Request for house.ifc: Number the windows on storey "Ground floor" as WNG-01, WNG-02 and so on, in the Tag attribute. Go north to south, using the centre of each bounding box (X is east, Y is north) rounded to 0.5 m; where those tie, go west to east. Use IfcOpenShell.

First a look at what the model holds.

```python
import ifcopenshell
import ifcopenshell.util.element
import ifcopenshell.util.placement

model = ifcopenshell.open("house.ifc")
print(model.schema)
storey = next(s for s in model.by_type("IfcBuildingStorey") if s.Name == "Ground floor")
windows = [e for e in ifcopenshell.util.element.get_decomposition(storey) if e.is_a("IfcWindow")]
for e in sorted(windows, key=lambda e: e.id()):
    origin = ifcopenshell.util.placement.get_local_placement(e.ObjectPlacement)[:3, 3]
    print(e.id(), e.Tag, e.Name, origin.round(2) + 0.0, sep=" | ")
```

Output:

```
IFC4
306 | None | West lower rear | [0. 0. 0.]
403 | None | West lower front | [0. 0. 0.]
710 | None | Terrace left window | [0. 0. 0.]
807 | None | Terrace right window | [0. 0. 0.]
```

```python
import ifcopenshell
import ifcopenshell.geom
import ifcopenshell.util.element
import ifcopenshell.util.shape

model = ifcopenshell.open("house.ifc")
settings = ifcopenshell.geom.settings()
settings.set("use-world-coords", True)


def centre(element):
    shape = ifcopenshell.geom.create_shape(settings, element)
    return ifcopenshell.util.shape.get_bbox_centroid(shape.geometry)


storey = next(s for s in model.by_type("IfcBuildingStorey") if s.Name == "Ground floor")
windows = [e for e in ifcopenshell.util.element.get_decomposition(storey) if e.is_a("IfcWindow")]

# Insertion points can sit at a corner or the storey origin, so sort by the geometry (in metres).
centres = {e: centre(e) for e in windows}
windows.sort(key=lambda e: (-round(centres[e][1] / 0.5), centres[e][0]))

for i, e in enumerate(windows, start=1):
    number = f"WNG-{i:02d}"
    e.Tag = number
    print(e.id(), number)

model.write("house_rev.ifc")
```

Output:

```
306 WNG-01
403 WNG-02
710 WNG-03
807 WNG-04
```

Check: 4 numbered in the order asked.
